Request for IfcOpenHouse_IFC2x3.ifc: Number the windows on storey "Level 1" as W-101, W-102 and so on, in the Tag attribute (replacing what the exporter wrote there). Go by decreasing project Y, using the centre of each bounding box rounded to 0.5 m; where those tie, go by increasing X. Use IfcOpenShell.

First a look at what the model holds.

```python
import ifcopenshell
import ifcopenshell.util.element
import ifcopenshell.util.placement

model = ifcopenshell.open("IfcOpenHouse_IFC2x3.ifc")
print(model.schema)
storey = next(s for s in model.by_type("IfcBuildingStorey") if s.Name == "Level 1")
windows = [e for e in ifcopenshell.util.element.get_decomposition(storey) if e.is_a("IfcWindow")]
for e in sorted(windows, key=lambda e: e.id()):
    origin = ifcopenshell.util.placement.get_local_placement(e.ObjectPlacement)[:3, 3]
    print(e.id(), e.Tag, e.Name, origin.round(2) + 0.0, sep=" | ")
```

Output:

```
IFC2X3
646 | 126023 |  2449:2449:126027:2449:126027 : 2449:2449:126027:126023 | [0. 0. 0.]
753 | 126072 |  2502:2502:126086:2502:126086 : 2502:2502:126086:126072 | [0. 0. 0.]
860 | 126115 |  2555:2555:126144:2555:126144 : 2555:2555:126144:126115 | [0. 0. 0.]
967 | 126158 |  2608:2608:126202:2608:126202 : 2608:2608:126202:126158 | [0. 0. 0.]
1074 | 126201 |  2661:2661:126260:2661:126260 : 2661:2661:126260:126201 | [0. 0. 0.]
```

```python
import ifcopenshell
import ifcopenshell.geom
import ifcopenshell.util.element
import ifcopenshell.util.shape

model = ifcopenshell.open("IfcOpenHouse_IFC2x3.ifc")
settings = ifcopenshell.geom.settings()
settings.set("use-world-coords", True)


def centre(element):
    shape = ifcopenshell.geom.create_shape(settings, element)
    return ifcopenshell.util.shape.get_bbox_centroid(shape.geometry)


storey = next(s for s in model.by_type("IfcBuildingStorey") if s.Name == "Level 1")
windows = [e for e in ifcopenshell.util.element.get_decomposition(storey) if e.is_a("IfcWindow")]

# Insertion points can sit at a corner or the storey origin, so sort by the geometry (in metres).
centres = {e: centre(e) for e in windows}
windows.sort(key=lambda e: (-round(centres[e][1] / 0.5), centres[e][0]))

for i, e in enumerate(windows, start=1):
    number = f"W-1{i:02d}"
    e.Tag = number
    print(e.id(), number)

model.write("IfcOpenHouse_IFC2x3_v2.ifc")
```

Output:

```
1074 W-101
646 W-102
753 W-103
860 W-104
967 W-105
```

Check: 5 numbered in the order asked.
